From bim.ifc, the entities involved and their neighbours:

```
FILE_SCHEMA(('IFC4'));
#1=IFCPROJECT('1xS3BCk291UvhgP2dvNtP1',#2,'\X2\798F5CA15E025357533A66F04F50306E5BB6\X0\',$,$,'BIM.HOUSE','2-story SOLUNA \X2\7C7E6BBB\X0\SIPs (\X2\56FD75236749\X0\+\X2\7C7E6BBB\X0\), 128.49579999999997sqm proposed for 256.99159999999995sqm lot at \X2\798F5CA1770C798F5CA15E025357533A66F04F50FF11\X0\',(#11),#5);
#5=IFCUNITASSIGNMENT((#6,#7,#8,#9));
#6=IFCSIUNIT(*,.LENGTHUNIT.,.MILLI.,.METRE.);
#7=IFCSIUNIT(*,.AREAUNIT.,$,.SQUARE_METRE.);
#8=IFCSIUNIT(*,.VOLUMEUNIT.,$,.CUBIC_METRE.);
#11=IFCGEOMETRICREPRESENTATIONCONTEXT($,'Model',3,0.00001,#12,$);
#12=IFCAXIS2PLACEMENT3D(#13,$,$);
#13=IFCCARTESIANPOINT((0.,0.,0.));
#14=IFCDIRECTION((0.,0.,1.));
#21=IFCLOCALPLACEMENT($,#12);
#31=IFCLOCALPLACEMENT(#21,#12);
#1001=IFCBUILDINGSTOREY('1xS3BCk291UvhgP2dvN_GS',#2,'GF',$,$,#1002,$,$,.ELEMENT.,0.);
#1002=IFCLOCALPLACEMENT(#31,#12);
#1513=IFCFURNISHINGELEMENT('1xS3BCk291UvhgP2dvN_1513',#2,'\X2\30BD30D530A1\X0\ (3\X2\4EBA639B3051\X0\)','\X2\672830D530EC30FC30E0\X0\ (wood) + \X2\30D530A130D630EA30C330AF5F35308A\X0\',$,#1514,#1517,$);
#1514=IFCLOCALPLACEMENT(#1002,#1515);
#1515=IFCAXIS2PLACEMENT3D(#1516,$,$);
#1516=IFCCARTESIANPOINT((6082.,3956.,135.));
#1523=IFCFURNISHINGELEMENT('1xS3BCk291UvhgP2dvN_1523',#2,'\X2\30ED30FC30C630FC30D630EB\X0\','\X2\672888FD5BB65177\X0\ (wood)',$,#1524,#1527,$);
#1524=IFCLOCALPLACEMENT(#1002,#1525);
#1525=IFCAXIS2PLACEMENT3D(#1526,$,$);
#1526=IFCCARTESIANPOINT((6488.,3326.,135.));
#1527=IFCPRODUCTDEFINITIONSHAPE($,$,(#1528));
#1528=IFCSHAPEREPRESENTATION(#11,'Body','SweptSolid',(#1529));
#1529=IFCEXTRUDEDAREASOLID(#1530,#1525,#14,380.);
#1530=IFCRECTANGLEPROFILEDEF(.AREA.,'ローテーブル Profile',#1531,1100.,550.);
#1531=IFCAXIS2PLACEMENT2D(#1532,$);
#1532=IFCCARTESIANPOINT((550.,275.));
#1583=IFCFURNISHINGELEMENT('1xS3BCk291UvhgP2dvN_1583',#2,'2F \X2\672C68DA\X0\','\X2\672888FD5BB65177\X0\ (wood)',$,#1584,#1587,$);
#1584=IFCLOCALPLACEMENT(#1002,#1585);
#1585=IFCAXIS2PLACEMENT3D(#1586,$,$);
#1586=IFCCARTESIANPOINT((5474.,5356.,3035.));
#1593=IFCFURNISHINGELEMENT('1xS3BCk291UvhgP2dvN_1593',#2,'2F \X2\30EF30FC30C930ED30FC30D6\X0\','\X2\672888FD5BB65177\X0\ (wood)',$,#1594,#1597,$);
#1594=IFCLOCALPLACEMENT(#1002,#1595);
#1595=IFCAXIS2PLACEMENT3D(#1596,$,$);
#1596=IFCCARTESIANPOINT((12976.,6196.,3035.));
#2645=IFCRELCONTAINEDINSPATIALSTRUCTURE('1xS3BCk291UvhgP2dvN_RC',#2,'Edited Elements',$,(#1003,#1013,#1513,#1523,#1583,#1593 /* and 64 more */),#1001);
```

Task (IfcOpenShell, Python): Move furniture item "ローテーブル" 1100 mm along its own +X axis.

```python
import ifcopenshell
import ifcopenshell.api.geometry
import ifcopenshell.util.placement

model = ifcopenshell.open("bim.ifc")

item = model.by_guid("1xS3BCk291UvhgP2dvN_1523")
matrix = ifcopenshell.util.placement.get_local_placement(item.ObjectPlacement)
matrix[:3, 3] += matrix[:3, 0] * 1100.0
ifcopenshell.api.geometry.edit_object_placement(model, product=item, matrix=matrix, is_si=False)

print(ifcopenshell.util.placement.get_local_placement(item.ObjectPlacement).round(3) + 0.0)

model.write("bim_edited.ifc")
```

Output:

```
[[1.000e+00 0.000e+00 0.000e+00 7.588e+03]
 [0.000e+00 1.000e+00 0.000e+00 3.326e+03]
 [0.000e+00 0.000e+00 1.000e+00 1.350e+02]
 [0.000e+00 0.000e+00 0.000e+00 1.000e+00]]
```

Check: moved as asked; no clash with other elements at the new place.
